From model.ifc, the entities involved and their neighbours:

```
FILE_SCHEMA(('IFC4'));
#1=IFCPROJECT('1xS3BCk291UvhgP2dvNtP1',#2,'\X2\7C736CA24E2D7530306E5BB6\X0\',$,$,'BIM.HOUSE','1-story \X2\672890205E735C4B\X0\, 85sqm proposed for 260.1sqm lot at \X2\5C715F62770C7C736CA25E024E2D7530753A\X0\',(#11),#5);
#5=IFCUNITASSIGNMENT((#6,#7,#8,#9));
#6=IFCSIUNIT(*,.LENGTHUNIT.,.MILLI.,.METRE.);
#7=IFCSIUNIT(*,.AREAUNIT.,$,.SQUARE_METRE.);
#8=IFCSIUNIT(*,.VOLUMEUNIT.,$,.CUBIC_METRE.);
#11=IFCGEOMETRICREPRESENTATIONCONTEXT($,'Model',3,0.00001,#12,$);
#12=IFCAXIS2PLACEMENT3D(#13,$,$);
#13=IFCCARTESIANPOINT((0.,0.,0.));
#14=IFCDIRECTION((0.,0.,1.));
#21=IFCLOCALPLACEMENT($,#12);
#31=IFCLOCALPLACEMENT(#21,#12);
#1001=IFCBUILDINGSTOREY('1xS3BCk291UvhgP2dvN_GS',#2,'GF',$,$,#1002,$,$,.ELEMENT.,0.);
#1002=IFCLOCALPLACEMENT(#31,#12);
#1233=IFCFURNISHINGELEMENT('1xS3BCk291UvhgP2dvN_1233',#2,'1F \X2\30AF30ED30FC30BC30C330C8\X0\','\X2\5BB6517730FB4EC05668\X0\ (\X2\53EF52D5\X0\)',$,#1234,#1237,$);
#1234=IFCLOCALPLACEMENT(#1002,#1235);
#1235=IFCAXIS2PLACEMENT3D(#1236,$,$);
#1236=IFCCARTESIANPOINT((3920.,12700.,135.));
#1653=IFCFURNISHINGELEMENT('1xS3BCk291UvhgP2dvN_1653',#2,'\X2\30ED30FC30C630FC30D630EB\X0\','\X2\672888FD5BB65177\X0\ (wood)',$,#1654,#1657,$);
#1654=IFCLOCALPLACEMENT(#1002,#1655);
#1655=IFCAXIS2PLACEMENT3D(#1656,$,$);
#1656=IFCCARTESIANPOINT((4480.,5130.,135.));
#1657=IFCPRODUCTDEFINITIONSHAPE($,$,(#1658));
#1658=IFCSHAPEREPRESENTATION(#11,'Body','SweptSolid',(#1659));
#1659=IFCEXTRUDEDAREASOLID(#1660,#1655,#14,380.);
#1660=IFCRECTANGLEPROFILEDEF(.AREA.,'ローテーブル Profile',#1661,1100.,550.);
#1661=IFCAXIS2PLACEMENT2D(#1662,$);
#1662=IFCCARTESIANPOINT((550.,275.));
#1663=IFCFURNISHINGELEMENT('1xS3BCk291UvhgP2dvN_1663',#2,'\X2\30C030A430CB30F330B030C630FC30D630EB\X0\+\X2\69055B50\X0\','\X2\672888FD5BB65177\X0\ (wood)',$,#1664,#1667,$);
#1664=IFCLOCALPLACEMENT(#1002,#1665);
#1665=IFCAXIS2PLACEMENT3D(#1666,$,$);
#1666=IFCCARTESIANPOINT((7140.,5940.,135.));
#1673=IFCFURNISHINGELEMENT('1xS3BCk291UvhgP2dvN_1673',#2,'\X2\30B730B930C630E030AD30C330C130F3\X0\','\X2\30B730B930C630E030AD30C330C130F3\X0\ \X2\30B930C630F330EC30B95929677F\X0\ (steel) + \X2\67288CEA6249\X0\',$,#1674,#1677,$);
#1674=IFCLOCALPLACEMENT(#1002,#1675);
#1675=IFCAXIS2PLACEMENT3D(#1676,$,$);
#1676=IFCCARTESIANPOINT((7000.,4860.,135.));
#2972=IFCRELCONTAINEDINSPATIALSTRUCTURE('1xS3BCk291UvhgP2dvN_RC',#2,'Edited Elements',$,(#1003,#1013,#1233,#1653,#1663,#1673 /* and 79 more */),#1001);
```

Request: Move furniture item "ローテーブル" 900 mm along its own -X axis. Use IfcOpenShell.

```python
import ifcopenshell
import ifcopenshell.api.geometry
import ifcopenshell.util.placement
import ifcopenshell.util.unit

model = ifcopenshell.open("model.ifc")
unit_scale = ifcopenshell.util.unit.calculate_unit_scale(model)

item = model.by_guid("1xS3BCk291UvhgP2dvN_1653")
matrix = ifcopenshell.util.placement.get_local_placement(item.ObjectPlacement)
matrix[:3, 3] -= matrix[:3, 0] * 0.9 / unit_scale
ifcopenshell.api.geometry.edit_object_placement(model, product=item, matrix=matrix, is_si=False)

print(ifcopenshell.util.placement.get_local_placement(item.ObjectPlacement).round(3) + 0.0)

model.write("model_updated.ifc")
```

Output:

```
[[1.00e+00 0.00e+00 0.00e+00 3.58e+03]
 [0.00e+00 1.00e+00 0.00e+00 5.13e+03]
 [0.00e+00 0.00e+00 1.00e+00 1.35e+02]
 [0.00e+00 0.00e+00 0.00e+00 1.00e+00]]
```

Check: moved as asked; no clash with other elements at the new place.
